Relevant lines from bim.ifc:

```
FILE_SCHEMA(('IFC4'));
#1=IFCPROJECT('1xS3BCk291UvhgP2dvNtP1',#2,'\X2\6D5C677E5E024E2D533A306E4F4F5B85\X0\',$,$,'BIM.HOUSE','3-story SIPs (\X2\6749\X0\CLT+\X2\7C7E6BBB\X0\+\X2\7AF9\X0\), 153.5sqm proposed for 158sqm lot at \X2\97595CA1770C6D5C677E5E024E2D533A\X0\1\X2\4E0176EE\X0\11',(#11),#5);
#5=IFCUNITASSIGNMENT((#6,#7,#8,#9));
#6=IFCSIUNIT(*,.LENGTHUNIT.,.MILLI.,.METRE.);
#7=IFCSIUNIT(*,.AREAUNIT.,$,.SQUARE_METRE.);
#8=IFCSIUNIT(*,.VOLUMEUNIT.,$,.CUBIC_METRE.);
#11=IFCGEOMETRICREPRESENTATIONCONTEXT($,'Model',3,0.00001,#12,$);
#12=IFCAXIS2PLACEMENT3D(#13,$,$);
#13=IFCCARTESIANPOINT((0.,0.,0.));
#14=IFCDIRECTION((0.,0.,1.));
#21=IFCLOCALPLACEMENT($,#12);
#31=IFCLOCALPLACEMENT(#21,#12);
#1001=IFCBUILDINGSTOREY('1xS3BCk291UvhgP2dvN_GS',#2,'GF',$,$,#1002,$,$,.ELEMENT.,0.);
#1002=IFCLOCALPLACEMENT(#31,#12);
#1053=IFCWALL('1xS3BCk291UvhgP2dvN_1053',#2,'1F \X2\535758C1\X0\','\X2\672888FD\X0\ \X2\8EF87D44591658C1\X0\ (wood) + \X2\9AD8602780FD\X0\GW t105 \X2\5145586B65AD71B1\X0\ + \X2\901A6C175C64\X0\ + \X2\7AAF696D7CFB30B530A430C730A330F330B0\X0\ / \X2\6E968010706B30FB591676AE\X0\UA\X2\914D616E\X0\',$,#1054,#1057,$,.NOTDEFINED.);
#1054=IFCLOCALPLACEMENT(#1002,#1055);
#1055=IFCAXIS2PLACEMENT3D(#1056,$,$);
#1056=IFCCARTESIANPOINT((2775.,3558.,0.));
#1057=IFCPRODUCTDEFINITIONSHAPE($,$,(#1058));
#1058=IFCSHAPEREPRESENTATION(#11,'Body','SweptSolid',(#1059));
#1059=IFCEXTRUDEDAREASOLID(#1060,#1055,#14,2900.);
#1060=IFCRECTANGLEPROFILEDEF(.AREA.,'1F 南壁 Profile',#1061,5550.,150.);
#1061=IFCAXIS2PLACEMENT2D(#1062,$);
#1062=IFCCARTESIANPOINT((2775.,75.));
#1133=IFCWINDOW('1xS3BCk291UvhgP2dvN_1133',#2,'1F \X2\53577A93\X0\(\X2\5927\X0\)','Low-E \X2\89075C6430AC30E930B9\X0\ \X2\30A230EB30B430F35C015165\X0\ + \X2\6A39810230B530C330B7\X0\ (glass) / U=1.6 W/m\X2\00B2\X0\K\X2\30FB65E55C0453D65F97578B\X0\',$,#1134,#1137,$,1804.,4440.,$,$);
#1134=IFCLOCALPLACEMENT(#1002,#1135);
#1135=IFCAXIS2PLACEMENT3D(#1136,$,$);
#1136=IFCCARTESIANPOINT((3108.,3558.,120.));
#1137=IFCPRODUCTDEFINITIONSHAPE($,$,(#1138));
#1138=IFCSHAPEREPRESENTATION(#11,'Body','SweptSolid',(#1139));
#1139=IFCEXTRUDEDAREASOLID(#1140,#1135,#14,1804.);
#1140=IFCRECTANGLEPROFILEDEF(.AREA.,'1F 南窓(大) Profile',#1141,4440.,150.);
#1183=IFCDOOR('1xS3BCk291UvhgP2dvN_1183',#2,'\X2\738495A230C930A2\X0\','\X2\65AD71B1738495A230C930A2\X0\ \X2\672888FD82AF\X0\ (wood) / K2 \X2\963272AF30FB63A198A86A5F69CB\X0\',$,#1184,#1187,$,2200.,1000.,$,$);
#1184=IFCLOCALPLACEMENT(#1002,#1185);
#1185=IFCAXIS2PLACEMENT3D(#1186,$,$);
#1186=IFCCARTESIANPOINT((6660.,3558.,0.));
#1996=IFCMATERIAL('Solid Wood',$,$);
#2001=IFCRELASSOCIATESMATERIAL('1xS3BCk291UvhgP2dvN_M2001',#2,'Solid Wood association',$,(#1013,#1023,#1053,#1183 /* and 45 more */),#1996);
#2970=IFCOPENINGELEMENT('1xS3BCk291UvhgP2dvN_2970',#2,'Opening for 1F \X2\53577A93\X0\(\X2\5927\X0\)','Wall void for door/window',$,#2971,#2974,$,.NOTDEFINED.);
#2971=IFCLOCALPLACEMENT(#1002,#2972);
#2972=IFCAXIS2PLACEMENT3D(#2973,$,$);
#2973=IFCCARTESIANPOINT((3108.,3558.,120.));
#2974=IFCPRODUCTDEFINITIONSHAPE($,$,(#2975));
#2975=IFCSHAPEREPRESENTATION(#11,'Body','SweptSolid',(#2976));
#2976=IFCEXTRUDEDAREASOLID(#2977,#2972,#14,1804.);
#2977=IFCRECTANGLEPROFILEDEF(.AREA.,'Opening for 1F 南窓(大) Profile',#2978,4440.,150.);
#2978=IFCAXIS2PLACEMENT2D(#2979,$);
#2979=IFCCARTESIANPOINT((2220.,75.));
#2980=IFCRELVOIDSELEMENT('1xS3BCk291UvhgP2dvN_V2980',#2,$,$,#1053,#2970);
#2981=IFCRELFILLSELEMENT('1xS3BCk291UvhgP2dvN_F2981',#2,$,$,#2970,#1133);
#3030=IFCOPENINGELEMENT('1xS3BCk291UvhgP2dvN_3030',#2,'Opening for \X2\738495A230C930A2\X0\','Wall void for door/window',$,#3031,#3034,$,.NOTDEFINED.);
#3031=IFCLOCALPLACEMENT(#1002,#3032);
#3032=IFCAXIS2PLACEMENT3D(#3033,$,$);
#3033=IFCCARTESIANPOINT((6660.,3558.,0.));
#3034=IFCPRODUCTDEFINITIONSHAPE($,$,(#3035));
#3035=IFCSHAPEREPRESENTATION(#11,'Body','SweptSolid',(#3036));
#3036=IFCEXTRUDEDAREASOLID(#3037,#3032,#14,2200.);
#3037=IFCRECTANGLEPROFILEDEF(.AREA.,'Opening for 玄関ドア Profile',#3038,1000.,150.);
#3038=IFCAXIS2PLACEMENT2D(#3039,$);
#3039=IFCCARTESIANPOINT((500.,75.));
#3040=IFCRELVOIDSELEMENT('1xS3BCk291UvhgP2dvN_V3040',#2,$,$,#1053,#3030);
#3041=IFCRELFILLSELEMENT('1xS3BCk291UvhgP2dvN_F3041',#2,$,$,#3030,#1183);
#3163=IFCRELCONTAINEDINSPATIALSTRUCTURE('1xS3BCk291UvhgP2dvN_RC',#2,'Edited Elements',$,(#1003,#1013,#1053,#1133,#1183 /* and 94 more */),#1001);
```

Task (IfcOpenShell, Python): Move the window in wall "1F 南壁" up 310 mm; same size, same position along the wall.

```python
import numpy as np
import ifcopenshell
import ifcopenshell.api.geometry
import ifcopenshell.util.placement
import ifcopenshell.util.unit

model = ifcopenshell.open("bim.ifc")
unit_scale = ifcopenshell.util.unit.calculate_unit_scale(model)

window = model.by_guid("1xS3BCk291UvhgP2dvN_1133")
opening = window.FillsVoids[0].RelatingOpeningElement
dz = 310.0

shift = np.array([0.0, 0.0, dz])
# The window is not placed relative to its opening, so move both.
for product in (opening, window):
    matrix = ifcopenshell.util.placement.get_local_placement(product.ObjectPlacement)
    matrix[:3, 3] += shift
    ifcopenshell.api.geometry.edit_object_placement(model, product=product, matrix=matrix, is_si=False)

print(f"moved by {dz * unit_scale:+.3f} m")

model.write("bim_updated.ifc")
```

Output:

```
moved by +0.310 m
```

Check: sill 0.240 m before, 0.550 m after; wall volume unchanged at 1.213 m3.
